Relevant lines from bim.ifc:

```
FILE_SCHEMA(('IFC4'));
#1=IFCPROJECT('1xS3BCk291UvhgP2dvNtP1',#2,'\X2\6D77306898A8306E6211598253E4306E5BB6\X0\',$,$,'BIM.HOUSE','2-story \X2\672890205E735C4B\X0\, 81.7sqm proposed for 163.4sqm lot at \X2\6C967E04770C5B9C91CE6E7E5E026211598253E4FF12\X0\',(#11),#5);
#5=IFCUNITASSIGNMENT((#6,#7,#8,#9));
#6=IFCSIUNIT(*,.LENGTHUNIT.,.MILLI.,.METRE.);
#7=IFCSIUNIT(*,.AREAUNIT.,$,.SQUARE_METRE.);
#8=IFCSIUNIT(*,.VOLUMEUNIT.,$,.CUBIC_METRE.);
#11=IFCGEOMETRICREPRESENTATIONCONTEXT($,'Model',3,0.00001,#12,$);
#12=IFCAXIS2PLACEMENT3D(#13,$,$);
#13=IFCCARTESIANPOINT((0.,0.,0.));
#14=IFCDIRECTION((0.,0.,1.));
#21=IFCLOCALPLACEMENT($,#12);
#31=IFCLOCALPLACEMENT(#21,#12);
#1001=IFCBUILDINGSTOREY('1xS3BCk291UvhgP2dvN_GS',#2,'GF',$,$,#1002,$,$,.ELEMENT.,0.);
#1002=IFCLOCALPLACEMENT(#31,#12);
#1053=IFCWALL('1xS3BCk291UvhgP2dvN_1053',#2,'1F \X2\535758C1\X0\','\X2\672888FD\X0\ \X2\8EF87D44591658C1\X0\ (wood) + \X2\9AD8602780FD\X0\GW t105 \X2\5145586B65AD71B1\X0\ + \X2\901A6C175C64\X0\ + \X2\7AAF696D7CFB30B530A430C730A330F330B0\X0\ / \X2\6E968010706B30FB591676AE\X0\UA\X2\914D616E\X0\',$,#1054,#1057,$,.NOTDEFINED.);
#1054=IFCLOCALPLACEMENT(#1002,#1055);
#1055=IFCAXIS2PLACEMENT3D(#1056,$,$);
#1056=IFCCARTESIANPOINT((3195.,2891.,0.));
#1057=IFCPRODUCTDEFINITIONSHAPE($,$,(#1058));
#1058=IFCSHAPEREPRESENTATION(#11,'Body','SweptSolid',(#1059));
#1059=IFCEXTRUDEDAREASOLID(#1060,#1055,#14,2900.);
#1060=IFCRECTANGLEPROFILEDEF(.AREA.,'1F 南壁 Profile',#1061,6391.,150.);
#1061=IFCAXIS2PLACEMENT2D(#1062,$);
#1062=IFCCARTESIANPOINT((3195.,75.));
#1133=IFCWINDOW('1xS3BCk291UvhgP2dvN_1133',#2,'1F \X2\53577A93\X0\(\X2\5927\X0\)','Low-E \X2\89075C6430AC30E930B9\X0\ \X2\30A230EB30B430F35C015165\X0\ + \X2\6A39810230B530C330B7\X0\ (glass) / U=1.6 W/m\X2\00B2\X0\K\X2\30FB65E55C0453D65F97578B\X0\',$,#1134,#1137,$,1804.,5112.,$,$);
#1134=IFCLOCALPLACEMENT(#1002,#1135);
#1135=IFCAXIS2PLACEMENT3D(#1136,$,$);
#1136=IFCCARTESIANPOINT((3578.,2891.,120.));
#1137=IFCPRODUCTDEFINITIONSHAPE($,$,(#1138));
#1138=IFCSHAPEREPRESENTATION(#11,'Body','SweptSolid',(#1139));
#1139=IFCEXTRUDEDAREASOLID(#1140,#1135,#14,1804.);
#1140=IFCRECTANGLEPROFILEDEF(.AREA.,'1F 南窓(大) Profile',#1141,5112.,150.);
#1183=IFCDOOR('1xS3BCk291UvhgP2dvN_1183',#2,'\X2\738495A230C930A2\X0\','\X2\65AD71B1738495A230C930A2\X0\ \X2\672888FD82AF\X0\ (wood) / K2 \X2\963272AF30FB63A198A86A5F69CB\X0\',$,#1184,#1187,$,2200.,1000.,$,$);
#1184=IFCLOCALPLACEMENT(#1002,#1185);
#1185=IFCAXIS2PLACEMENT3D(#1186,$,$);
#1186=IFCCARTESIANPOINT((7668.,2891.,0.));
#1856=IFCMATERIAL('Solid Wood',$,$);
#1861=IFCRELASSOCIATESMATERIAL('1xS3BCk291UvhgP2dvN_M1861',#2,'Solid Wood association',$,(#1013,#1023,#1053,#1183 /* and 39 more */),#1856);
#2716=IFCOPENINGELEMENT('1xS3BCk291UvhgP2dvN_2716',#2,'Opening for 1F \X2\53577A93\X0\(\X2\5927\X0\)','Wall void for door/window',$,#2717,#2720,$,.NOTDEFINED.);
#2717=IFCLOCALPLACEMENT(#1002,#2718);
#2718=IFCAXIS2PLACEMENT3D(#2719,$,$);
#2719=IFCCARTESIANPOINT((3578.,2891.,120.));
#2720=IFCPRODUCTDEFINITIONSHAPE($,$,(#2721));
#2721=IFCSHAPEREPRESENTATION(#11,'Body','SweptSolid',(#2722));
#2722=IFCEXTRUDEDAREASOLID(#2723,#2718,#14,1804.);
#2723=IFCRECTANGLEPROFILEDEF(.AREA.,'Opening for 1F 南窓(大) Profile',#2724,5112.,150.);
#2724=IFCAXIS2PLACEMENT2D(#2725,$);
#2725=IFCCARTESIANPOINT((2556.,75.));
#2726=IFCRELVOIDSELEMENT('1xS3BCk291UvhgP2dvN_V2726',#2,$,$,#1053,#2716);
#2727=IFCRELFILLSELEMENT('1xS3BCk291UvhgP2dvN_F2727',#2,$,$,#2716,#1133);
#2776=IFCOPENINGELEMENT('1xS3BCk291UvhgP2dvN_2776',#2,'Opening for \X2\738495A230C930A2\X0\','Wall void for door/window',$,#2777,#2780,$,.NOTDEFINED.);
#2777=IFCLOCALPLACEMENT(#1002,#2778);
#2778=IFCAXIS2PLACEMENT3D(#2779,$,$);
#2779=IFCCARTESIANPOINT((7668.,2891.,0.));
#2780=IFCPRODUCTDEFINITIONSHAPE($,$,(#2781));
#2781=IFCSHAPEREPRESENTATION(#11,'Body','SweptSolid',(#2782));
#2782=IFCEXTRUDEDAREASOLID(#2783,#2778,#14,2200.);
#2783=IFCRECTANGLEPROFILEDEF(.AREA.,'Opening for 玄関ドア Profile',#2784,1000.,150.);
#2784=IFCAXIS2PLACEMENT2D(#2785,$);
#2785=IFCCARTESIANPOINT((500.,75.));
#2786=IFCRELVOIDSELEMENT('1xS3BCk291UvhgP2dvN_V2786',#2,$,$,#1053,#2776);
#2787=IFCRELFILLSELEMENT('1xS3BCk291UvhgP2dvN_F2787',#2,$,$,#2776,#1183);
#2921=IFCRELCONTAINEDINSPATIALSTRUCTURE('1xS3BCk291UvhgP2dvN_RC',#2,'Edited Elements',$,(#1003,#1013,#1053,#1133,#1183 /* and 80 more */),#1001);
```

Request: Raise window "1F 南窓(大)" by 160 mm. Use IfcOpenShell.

```python
import numpy as np
import ifcopenshell
import ifcopenshell.api.geometry
import ifcopenshell.util.placement
import ifcopenshell.util.unit

model = ifcopenshell.open("bim.ifc")
unit_scale = ifcopenshell.util.unit.calculate_unit_scale(model)

window = model.by_guid("1xS3BCk291UvhgP2dvN_1133")
opening = window.FillsVoids[0].RelatingOpeningElement
dz = 0.16 / unit_scale

shift = np.array([0.0, 0.0, dz])
# The window is not placed relative to its opening, so move both.
for product in (opening, window):
    matrix = ifcopenshell.util.placement.get_local_placement(product.ObjectPlacement)
    matrix[:3, 3] += shift
    ifcopenshell.api.geometry.edit_object_placement(model, product=product, matrix=matrix, is_si=False)

print(f"moved by {dz * unit_scale:+.3f} m")

model.write("bim_v2.ifc")
```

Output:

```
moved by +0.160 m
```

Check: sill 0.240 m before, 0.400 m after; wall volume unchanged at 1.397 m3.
